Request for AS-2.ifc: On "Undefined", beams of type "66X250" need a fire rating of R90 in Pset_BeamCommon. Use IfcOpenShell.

First a look at what the model holds.

```python
import ifcopenshell
import ifcopenshell.util.element

model = ifcopenshell.open("AS-2.ifc")
print(model.schema)
storey = next(s for s in model.by_type("IfcBuildingStorey") if s.Name == "Undefined")
beams = [e for e in ifcopenshell.util.element.get_decomposition(storey) if e.is_a("IfcBeam")]
seen = {}
for e in beams:
    element_type = ifcopenshell.util.element.get_type(e)
    key = (element_type.Name if element_type != e and element_type else None, ifcopenshell.util.element.get_pset(e, "Pset_BeamCommon", "FireRating"))
    seen[key] = seen.get(key, 0) + 1
for (name, value), count in sorted(seen.items(), key=str):
    print(count, "x", name, "|", value)
```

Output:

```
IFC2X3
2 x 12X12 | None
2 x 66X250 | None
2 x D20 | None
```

```python
import ifcopenshell
import ifcopenshell.api.pset
import ifcopenshell.util.element

model = ifcopenshell.open("AS-2.ifc")

storey = next(s for s in model.by_type("IfcBuildingStorey") if s.Name == "Undefined")
beams = [e for e in ifcopenshell.util.element.get_decomposition(storey) if e.is_a("IfcBeam")]

count = 0
for e in beams:
    element_type = ifcopenshell.util.element.get_type(e)
    if element_type in (None, e) or element_type.Name != "66X250":
        continue
    found = ifcopenshell.util.element.get_pset(e, "Pset_BeamCommon", should_inherit=False)
    if found:
        pset = model.by_id(found["id"])
        if len(ifcopenshell.util.element.get_elements_by_pset(pset)) > 1:
            pset = ifcopenshell.api.pset.unshare_pset(model, products=[e], pset=pset)[0]
    else:
        pset = ifcopenshell.api.pset.add_pset(model, product=e, name="Pset_BeamCommon")
    ifcopenshell.api.pset.edit_pset(model, pset=pset, properties={"FireRating": "R90"})
    count += 1

print(count, "beams updated")

model.write("AS-2-out.ifc")
```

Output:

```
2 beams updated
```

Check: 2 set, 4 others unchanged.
